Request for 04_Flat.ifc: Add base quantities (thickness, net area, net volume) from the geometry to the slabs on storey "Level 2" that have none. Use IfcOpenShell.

First a look at what the model holds.

```python
import ifcopenshell
import ifcopenshell.util.element
import ifcopenshell.util.unit

model = ifcopenshell.open("04_Flat.ifc")
print(model.schema)
for unit_type in ("LENGTHUNIT", "AREAUNIT", "VOLUMEUNIT"):
    print(unit_type, ifcopenshell.util.unit.calculate_unit_scale(model, unit_type))
storey = next(s for s in model.by_type("IfcBuildingStorey") if s.Name == "Level 2")
slabs = [e for e in ifcopenshell.util.element.get_decomposition(storey) if e.is_a("IfcSlab")]
for e in sorted(slabs, key=lambda e: e.id()):
    print(e.id(), e.is_a(), e.Name, list(ifcopenshell.util.element.get_psets(e, qtos_only=True)), sep=" | ")
```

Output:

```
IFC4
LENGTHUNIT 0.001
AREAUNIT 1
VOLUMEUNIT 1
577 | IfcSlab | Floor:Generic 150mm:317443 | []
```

```python
import ifcopenshell
import ifcopenshell.api.pset
import ifcopenshell.geom
import ifcopenshell.util.element
import ifcopenshell.util.shape
import ifcopenshell.util.unit

model = ifcopenshell.open("04_Flat.ifc")
unit_scale = ifcopenshell.util.unit.calculate_unit_scale(model)
area_scale = ifcopenshell.util.unit.calculate_unit_scale(model, "AREAUNIT")
volume_scale = ifcopenshell.util.unit.calculate_unit_scale(model, "VOLUMEUNIT")
settings = ifcopenshell.geom.settings()

storey = next(s for s in model.by_type("IfcBuildingStorey") if s.Name == "Level 2")
slabs = [e for e in ifcopenshell.util.element.get_decomposition(storey) if e.is_a("IfcSlab")]

for e in sorted(slabs, key=lambda e: e.id()):
    if ifcopenshell.util.element.get_psets(e, qtos_only=True, should_inherit=False):
        continue
    # Geometry comes back in metres, in the element's own axes.
    shape = ifcopenshell.geom.create_shape(settings, e)
    values = {
        "Width": ifcopenshell.util.shape.get_z(shape.geometry) / unit_scale,
        "NetArea": ifcopenshell.util.shape.get_footprint_area(shape.geometry) / area_scale,
        "NetVolume": ifcopenshell.util.shape.get_volume(shape.geometry) / volume_scale,
    }
    qto = ifcopenshell.api.pset.add_qto(model, product=e, name="Qto_SlabBaseQuantities")
    ifcopenshell.api.pset.edit_qto(model, qto=qto, properties=values)
    print(e.id(), {k: round(v, 3) for k, v in values.items()})

model.write("04_Flat_edited.ifc")
```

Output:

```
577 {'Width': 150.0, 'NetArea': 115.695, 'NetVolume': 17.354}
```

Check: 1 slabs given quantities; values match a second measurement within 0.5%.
